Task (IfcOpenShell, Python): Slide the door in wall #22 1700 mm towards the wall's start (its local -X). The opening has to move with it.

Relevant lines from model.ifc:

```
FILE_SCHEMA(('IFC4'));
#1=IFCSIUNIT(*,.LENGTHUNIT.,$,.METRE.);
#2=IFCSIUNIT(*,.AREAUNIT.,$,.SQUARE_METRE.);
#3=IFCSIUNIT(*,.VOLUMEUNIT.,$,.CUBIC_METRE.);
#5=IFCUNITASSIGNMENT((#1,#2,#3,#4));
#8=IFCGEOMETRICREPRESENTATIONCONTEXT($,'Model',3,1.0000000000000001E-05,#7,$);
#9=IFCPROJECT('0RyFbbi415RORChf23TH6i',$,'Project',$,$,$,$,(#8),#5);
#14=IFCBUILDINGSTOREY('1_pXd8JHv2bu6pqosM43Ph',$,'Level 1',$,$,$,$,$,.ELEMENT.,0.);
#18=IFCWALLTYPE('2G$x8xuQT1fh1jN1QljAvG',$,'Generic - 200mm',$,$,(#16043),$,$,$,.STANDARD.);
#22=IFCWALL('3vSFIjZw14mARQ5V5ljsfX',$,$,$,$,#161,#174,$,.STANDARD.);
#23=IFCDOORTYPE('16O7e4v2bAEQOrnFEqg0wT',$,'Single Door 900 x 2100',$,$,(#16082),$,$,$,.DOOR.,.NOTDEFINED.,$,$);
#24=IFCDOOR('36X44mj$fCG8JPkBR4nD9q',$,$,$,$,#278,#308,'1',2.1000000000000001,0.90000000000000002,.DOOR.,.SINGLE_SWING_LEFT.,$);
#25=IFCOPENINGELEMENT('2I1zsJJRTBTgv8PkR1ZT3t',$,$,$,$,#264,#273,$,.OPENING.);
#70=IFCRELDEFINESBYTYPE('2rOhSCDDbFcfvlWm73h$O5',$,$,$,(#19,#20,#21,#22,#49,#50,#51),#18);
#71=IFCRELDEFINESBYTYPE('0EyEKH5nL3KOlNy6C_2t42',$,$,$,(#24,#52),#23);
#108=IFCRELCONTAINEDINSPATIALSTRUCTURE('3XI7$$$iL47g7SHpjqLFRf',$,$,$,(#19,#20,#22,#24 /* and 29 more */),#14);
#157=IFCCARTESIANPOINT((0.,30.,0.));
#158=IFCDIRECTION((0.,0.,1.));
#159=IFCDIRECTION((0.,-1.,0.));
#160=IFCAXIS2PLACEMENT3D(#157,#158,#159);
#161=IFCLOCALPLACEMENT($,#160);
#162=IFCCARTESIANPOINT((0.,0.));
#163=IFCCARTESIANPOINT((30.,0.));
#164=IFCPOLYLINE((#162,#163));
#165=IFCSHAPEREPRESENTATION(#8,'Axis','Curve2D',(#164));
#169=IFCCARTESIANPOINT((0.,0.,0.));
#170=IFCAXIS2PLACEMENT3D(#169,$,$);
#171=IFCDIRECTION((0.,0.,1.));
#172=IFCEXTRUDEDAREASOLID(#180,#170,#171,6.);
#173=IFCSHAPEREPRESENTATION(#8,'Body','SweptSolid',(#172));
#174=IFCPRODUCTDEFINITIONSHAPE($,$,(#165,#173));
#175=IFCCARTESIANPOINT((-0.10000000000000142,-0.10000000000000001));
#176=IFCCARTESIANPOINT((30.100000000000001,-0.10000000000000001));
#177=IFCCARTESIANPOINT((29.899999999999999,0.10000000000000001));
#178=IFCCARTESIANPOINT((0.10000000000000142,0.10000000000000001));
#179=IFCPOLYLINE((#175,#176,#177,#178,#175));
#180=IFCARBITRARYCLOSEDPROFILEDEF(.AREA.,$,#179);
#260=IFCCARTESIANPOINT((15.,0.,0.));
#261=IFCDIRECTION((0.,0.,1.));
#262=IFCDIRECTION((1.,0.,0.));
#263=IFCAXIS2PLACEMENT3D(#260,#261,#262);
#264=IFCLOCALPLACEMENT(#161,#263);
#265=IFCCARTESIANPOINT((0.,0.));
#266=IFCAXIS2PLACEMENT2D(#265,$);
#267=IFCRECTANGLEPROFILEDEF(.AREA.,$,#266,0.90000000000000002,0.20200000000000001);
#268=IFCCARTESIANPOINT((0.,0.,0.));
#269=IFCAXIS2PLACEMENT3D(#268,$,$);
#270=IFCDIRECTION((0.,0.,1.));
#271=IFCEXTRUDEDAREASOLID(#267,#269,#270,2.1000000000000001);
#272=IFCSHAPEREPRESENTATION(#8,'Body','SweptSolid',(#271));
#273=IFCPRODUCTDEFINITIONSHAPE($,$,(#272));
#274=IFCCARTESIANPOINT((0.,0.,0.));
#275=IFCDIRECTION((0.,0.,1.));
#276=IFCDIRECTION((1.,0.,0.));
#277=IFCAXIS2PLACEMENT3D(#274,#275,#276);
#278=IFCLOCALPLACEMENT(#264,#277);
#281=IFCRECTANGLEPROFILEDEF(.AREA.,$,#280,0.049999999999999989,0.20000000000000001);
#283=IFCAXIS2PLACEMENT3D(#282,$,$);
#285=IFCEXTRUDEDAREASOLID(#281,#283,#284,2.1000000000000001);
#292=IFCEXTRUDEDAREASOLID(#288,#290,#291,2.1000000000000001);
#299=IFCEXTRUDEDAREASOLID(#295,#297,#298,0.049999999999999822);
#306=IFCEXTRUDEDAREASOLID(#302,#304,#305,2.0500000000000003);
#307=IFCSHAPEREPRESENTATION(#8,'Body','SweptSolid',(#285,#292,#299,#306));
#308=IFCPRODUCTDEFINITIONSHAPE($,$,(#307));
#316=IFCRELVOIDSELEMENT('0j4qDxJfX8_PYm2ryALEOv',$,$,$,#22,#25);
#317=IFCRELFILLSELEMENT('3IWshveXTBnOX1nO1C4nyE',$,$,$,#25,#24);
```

```python
import ifcopenshell
import ifcopenshell.api.geometry
import ifcopenshell.util.placement
import ifcopenshell.util.unit

model = ifcopenshell.open("model.ifc")
unit_scale = ifcopenshell.util.unit.calculate_unit_scale(model)

door = model.by_guid("36X44mj$fCG8JPkBR4nD9q")
opening = door.FillsVoids[0].RelatingOpeningElement
wall = opening.VoidsElements[0].RelatingBuildingElement

wall_matrix = ifcopenshell.util.placement.get_local_placement(wall.ObjectPlacement)
shift = wall_matrix[:3, 0] * -1.7 / unit_scale
before = ifcopenshell.util.placement.get_local_placement(door.ObjectPlacement)[:3, 3].copy()

# The door is placed relative to its opening, so it follows when the opening moves.
matrix = ifcopenshell.util.placement.get_local_placement(opening.ObjectPlacement)
matrix[:3, 3] += shift
ifcopenshell.api.geometry.edit_object_placement(
    model, product=opening, matrix=matrix, is_si=False, should_transform_children=True
)

after = ifcopenshell.util.placement.get_local_placement(door.ObjectPlacement)[:3, 3]
print("door moved by", (after - before).round(3) + 0.0)

model.write("model_edited.ifc")
```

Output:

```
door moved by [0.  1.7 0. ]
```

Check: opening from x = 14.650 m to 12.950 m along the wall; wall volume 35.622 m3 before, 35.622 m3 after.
